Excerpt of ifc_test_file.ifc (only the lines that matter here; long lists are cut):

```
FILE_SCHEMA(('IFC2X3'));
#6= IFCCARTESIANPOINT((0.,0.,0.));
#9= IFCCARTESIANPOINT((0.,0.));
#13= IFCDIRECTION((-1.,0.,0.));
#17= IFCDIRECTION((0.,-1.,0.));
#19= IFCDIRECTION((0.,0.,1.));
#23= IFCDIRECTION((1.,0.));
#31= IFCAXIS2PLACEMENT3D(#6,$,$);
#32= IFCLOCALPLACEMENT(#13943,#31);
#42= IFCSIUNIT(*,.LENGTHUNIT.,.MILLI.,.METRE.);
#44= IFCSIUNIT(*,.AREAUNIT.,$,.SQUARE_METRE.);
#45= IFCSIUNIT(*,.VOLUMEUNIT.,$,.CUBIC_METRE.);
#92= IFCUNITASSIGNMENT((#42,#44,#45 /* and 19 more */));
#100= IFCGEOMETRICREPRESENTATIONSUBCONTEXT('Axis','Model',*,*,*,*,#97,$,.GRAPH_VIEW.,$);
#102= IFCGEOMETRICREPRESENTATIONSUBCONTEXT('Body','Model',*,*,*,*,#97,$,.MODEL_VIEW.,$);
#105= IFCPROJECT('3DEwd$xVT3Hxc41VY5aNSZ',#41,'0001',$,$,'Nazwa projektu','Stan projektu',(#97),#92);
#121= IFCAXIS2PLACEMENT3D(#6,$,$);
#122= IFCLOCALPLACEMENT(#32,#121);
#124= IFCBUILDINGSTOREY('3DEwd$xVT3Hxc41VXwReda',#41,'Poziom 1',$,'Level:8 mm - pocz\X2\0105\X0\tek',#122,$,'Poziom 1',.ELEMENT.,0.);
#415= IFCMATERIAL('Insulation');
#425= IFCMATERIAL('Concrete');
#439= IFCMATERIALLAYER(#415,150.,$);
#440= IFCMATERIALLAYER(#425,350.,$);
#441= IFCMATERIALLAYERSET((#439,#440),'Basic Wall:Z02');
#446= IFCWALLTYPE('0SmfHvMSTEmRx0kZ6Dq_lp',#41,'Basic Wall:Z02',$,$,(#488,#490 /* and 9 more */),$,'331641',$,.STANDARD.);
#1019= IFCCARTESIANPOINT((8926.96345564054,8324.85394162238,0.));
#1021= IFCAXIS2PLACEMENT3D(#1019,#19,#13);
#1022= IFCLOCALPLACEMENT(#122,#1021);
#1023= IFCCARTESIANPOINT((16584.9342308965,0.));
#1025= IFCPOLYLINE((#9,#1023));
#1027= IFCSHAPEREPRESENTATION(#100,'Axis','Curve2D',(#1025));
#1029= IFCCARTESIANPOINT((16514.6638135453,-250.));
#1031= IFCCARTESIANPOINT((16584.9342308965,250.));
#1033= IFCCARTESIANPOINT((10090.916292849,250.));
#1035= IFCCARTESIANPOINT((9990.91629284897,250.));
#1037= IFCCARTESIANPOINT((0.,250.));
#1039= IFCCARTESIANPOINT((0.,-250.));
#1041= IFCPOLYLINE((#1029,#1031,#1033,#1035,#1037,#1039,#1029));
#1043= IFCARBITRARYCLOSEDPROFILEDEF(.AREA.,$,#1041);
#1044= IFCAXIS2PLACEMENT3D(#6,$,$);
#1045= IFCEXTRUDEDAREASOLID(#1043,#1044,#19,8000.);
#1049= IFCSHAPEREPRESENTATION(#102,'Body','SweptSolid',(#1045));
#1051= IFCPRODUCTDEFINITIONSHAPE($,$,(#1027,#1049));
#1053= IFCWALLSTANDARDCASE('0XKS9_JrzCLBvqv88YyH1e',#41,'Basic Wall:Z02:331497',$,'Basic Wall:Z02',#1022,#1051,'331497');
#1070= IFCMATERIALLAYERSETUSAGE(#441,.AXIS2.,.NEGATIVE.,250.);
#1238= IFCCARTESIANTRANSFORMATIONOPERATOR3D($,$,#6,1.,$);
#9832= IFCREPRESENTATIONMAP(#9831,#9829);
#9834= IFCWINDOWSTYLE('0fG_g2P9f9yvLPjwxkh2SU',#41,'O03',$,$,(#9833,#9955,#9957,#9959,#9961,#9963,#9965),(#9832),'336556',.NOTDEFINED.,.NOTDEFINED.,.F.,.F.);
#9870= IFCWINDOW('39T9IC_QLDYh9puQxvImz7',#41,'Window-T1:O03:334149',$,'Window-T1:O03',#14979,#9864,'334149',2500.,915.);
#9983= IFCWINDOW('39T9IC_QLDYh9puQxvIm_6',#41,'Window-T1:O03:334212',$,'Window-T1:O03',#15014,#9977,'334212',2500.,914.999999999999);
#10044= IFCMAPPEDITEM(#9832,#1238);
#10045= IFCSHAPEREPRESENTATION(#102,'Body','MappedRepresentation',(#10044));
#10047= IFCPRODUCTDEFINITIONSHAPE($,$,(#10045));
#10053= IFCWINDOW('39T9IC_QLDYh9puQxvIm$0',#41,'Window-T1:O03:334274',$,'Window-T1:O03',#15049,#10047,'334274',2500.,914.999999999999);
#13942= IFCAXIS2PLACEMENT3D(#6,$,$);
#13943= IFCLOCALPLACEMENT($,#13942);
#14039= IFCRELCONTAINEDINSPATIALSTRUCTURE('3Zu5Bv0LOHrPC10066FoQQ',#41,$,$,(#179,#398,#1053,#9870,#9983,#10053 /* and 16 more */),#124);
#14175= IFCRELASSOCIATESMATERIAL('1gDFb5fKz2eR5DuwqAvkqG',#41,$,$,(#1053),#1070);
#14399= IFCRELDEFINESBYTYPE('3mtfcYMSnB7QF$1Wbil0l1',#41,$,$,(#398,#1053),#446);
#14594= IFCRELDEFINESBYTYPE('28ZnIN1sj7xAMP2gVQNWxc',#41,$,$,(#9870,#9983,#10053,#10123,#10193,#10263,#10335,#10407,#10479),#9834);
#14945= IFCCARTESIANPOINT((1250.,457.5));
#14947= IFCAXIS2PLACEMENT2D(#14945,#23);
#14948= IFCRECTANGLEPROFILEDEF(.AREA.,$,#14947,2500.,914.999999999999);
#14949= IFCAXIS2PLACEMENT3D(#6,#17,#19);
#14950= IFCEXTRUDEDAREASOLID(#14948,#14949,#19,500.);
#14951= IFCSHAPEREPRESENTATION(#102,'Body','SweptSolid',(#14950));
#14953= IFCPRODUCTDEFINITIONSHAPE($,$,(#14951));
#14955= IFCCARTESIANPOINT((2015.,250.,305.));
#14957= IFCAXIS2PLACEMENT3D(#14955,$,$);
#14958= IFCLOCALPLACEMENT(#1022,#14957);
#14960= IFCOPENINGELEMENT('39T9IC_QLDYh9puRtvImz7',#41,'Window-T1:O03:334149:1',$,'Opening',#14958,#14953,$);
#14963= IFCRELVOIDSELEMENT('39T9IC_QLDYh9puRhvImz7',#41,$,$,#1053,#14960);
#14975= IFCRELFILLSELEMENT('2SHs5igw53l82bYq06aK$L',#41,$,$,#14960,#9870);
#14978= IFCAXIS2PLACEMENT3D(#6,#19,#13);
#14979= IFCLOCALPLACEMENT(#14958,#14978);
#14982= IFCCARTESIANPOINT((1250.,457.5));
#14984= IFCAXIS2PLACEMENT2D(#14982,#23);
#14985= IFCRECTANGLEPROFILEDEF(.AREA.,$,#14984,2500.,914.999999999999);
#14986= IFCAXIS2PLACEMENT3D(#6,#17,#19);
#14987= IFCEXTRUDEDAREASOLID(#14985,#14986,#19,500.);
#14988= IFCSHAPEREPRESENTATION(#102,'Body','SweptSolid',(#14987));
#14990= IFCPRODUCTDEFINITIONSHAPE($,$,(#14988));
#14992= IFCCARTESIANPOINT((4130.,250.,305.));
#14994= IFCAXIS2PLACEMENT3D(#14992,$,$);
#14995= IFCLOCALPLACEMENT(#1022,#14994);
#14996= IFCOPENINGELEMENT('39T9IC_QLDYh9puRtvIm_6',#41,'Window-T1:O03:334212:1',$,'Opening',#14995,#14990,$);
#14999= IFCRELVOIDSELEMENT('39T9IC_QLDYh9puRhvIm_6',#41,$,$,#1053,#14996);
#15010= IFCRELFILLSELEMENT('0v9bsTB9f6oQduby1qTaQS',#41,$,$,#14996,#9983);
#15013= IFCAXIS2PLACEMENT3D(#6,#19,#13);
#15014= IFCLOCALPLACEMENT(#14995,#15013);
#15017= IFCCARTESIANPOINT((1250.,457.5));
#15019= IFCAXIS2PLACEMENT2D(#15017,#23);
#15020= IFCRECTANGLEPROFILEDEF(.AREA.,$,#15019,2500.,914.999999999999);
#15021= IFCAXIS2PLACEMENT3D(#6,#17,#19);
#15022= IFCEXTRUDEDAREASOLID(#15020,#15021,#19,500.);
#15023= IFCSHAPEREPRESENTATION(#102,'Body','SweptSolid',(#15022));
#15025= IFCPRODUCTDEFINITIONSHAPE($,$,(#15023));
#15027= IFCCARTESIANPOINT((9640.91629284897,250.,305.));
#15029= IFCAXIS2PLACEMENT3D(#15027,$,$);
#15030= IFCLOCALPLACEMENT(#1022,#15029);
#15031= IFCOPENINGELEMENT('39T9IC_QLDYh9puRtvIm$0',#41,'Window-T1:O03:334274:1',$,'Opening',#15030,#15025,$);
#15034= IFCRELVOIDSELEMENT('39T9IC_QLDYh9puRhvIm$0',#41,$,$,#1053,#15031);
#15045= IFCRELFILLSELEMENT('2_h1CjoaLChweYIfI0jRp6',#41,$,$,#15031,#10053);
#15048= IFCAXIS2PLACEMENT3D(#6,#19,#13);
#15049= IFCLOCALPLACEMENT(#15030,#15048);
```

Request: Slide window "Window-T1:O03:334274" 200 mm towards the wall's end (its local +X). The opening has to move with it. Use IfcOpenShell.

```python
import ifcopenshell
import ifcopenshell.api.geometry
import ifcopenshell.util.placement

model = ifcopenshell.open("ifc_test_file.ifc")

window = model.by_guid("39T9IC_QLDYh9puQxvIm$0")
opening = window.FillsVoids[0].RelatingOpeningElement
wall = opening.VoidsElements[0].RelatingBuildingElement

wall_matrix = ifcopenshell.util.placement.get_local_placement(wall.ObjectPlacement)
shift = wall_matrix[:3, 0] * 200.0
before = ifcopenshell.util.placement.get_local_placement(window.ObjectPlacement)[:3, 3].copy()

# The window is placed relative to its opening, so it follows when the opening moves.
matrix = ifcopenshell.util.placement.get_local_placement(opening.ObjectPlacement)
matrix[:3, 3] += shift
ifcopenshell.api.geometry.edit_object_placement(
    model, product=opening, matrix=matrix, is_si=False, should_transform_children=True
)

after = ifcopenshell.util.placement.get_local_placement(window.ObjectPlacement)[:3, 3]
print("window moved by", (after - before).round(3) + 0.0)

model.write("ifc_test_file_v2.ifc")
```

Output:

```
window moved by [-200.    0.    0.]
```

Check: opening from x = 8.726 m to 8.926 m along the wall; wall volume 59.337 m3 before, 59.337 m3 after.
